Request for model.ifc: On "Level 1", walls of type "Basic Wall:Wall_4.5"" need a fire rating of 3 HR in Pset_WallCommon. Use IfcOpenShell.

First a look at what the model holds.

```python
import ifcopenshell
import ifcopenshell.util.element

model = ifcopenshell.open("model.ifc")
print(model.schema)
storey = next(s for s in model.by_type("IfcBuildingStorey") if s.Name == "Level 1")
walls = [e for e in ifcopenshell.util.element.get_decomposition(storey) if e.is_a("IfcWall")]
seen = {}
for e in walls:
    element_type = ifcopenshell.util.element.get_type(e)
    key = (element_type.Name if element_type != e and element_type else None, ifcopenshell.util.element.get_pset(e, "Pset_WallCommon", "FireRating"))
    seen[key] = seen.get(key, 0) + 1
for (name, value), count in sorted(seen.items(), key=str):
    print(count, "x", name, "|", value)
```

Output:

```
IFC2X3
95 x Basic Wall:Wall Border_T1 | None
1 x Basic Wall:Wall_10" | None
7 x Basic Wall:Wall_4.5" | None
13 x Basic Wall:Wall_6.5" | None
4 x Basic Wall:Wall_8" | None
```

```python
import ifcopenshell
import ifcopenshell.api.pset
import ifcopenshell.util.element

model = ifcopenshell.open("model.ifc")

storey = next(s for s in model.by_type("IfcBuildingStorey") if s.Name == "Level 1")
walls = [e for e in ifcopenshell.util.element.get_decomposition(storey) if e.is_a("IfcWall")]

count = 0
for e in walls:
    element_type = ifcopenshell.util.element.get_type(e)
    if element_type in (None, e) or element_type.Name != 'Basic Wall:Wall_4.5"':
        continue
    # add_pset returns the element's existing set when there is one.
    pset = ifcopenshell.api.pset.add_pset(model, product=e, name="Pset_WallCommon")
    ifcopenshell.api.pset.edit_pset(model, pset=pset, properties={"FireRating": "3 HR"})
    count += 1

print(count, "walls updated")

model.write("model_v2.ifc")
```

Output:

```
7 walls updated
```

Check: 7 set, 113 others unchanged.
